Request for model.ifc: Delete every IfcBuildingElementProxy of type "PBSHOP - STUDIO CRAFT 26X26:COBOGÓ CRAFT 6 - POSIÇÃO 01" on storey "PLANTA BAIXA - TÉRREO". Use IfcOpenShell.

First a look at what the model holds.

```python
import ifcopenshell
import ifcopenshell.util.element

model = ifcopenshell.open("model.ifc")
print(model.schema)
storey = next(s for s in model.by_type("IfcBuildingStorey") if s.Name == "PLANTA BAIXA - TÉRREO")
proxies = [e for e in ifcopenshell.util.element.get_decomposition(storey) if e.is_a("IfcBuildingElementProxy")]
seen = {}
for e in proxies:
    element_type = ifcopenshell.util.element.get_type(e)
    name = element_type.Name if element_type not in (None, e) else None
    seen[name] = seen.get(name, 0) + 1
for name, count in sorted(seen.items(), key=str):
    print(count, "x", name)
```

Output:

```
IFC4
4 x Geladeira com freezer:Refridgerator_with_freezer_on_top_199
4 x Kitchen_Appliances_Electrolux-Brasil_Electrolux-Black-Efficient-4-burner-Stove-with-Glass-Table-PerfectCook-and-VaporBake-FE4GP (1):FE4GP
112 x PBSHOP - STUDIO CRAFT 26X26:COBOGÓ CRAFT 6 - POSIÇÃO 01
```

```python
import ifcopenshell
import ifcopenshell.api.root
import ifcopenshell.util.element

model = ifcopenshell.open("model.ifc")

storey = next(s for s in model.by_type("IfcBuildingStorey") if s.Name == "PLANTA BAIXA - TÉRREO")
proxies = [e for e in ifcopenshell.util.element.get_decomposition(storey) if e.is_a("IfcBuildingElementProxy")]
targets = [e for e in proxies if (t := ifcopenshell.util.element.get_type(e)) not in (None, e) and t.Name == "PBSHOP - STUDIO CRAFT 26X26:COBOGÓ CRAFT 6 - POSIÇÃO 01"]

for e in targets:
    ifcopenshell.api.root.remove_product(model, product=e)
print(len(targets), "removed")

model.write("model_rev.ifc")
```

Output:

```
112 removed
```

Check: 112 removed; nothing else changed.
